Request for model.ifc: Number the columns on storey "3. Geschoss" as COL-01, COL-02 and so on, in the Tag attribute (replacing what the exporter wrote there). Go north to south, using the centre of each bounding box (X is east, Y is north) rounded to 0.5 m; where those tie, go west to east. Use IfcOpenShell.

First a look at what the model holds.

```python
import ifcopenshell
import ifcopenshell.util.element
import ifcopenshell.util.placement

model = ifcopenshell.open("model.ifc")
print(model.schema)
storey = next(s for s in model.by_type("IfcBuildingStorey") if s.Name == "3. Geschoss")
columns = [e for e in ifcopenshell.util.element.get_decomposition(storey) if e.is_a("IfcColumn")]
for e in sorted(columns, key=lambda e: e.id()):
    origin = ifcopenshell.util.placement.get_local_placement(e.ObjectPlacement)[:3, 3]
    print(e.id(), e.Tag, e.Name, origin.round(2) + 0.0, sep=" | ")
```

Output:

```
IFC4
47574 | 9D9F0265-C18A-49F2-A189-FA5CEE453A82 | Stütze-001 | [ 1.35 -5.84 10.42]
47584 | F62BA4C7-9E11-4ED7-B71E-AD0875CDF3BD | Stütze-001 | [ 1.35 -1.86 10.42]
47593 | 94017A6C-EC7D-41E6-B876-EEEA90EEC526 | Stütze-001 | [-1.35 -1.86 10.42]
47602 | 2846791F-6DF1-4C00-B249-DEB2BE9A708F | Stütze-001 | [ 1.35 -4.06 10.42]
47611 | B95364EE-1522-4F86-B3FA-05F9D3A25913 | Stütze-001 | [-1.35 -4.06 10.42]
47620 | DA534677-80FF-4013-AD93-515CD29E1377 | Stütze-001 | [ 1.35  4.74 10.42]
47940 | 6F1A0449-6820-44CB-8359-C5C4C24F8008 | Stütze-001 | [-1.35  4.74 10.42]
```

```python
import ifcopenshell
import ifcopenshell.geom
import ifcopenshell.util.element
import ifcopenshell.util.shape

model = ifcopenshell.open("model.ifc")
settings = ifcopenshell.geom.settings()
settings.set("use-world-coords", True)


def centre(element):
    shape = ifcopenshell.geom.create_shape(settings, element)
    return ifcopenshell.util.shape.get_bbox_centroid(shape.geometry)


storey = next(s for s in model.by_type("IfcBuildingStorey") if s.Name == "3. Geschoss")
columns = [e for e in ifcopenshell.util.element.get_decomposition(storey) if e.is_a("IfcColumn")]

# Insertion points can sit at a corner or the storey origin, so sort by the geometry (in metres).
centres = {e: centre(e) for e in columns}
columns.sort(key=lambda e: (-round(centres[e][1] / 0.5), centres[e][0]))

for i, e in enumerate(columns, start=1):
    number = f"COL-{i:02d}"
    e.Tag = number
    print(e.id(), number)

model.write("model-out.ifc")
```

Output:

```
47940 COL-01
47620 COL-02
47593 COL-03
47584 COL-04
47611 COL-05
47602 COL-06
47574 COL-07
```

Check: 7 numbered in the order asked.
